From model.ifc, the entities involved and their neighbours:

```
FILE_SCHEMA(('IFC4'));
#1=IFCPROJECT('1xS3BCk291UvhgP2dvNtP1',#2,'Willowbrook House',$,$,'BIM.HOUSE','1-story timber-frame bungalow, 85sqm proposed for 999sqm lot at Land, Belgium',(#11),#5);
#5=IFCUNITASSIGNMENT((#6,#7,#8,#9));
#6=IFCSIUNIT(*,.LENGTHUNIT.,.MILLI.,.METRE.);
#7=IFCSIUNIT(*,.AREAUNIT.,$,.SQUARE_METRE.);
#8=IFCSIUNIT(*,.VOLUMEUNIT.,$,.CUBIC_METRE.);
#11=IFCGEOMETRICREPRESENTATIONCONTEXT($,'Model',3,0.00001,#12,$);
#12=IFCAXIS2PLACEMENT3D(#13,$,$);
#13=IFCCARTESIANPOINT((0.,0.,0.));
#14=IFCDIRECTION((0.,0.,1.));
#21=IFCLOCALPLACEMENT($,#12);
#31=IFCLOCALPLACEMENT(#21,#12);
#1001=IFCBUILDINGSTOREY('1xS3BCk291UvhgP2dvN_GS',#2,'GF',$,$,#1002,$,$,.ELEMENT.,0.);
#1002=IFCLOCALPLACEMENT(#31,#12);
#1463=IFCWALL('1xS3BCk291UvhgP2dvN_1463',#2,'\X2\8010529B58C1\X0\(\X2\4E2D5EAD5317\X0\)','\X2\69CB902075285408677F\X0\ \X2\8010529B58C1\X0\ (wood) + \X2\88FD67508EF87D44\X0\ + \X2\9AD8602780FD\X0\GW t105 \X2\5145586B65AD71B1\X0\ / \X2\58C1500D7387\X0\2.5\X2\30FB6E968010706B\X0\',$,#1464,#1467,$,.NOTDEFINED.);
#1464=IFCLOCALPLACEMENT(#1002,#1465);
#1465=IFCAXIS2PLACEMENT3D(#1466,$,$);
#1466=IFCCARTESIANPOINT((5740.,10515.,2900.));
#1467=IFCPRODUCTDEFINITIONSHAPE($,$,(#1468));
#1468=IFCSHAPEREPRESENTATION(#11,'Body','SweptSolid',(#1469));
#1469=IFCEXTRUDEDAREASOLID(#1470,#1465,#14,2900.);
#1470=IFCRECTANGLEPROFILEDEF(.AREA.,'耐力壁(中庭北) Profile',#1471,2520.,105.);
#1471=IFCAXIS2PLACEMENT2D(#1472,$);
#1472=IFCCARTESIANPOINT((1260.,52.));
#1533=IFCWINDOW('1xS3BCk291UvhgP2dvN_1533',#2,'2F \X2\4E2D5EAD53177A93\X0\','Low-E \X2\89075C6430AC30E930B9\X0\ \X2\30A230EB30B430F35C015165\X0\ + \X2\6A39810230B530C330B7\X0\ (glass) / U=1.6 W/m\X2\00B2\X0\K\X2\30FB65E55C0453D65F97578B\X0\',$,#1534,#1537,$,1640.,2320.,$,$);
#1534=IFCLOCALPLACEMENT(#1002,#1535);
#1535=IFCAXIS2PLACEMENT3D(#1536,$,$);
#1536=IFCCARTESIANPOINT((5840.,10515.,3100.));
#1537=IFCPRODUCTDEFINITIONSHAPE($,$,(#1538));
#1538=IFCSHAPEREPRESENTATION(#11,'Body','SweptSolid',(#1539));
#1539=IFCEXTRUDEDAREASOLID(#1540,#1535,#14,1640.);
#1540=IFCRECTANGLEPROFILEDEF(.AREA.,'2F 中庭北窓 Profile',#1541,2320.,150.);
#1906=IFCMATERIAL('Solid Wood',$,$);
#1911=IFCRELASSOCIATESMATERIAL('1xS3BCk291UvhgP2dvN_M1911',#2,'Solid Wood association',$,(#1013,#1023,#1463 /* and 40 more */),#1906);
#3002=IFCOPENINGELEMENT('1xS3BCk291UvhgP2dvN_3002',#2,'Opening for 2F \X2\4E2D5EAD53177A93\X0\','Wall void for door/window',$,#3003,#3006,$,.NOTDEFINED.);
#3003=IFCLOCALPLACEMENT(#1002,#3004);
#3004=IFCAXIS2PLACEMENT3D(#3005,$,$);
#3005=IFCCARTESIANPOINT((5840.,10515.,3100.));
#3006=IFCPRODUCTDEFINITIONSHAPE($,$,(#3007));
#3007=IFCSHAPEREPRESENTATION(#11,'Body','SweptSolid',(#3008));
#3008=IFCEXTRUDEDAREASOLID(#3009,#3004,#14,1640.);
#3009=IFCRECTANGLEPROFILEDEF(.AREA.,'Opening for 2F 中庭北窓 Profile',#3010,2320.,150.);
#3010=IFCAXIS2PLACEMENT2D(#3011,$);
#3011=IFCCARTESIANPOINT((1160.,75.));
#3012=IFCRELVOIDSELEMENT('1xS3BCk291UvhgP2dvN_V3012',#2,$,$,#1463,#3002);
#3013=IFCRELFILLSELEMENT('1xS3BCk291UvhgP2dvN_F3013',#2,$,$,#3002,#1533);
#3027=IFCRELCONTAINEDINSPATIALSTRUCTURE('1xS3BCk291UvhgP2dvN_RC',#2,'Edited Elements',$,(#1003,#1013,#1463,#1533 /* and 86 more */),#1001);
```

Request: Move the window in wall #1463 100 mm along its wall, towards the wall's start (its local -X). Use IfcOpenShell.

```python
import ifcopenshell
import ifcopenshell.api.geometry
import ifcopenshell.util.placement

model = ifcopenshell.open("model.ifc")

window = model.by_id(1533)
opening = window.FillsVoids[0].RelatingOpeningElement
wall = opening.VoidsElements[0].RelatingBuildingElement

wall_matrix = ifcopenshell.util.placement.get_local_placement(wall.ObjectPlacement)
shift = wall_matrix[:3, 0] * -100.0
before = ifcopenshell.util.placement.get_local_placement(window.ObjectPlacement)[:3, 3].copy()

# The window is not placed relative to its opening, so move both.
for product in (opening, window):
    matrix = ifcopenshell.util.placement.get_local_placement(product.ObjectPlacement)
    matrix[:3, 3] += shift
    ifcopenshell.api.geometry.edit_object_placement(model, product=product, matrix=matrix, is_si=False)

after = ifcopenshell.util.placement.get_local_placement(window.ObjectPlacement)[:3, 3]
print("window moved by", (after - before).round(3) + 0.0)

model.write("model_v2.ifc")
```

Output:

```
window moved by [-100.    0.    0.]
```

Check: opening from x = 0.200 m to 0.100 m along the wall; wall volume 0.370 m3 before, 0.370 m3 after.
